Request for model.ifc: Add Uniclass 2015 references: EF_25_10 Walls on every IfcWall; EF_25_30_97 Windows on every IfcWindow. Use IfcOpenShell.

First a look at what the model holds.

```python
import ifcopenshell

model = ifcopenshell.open("model.ifc")
print(model.schema)
print("classifications:", [c.Name for c in model.by_type("IfcClassification")])
for ifc_class in ("IfcDoor", "IfcRoof", "IfcStair", "IfcWall", "IfcWindow"):
    print(ifc_class, len(model.by_type(ifc_class)))
```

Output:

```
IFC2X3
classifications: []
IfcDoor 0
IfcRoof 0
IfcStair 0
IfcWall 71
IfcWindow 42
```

```python
import ifcopenshell
import ifcopenshell.api.classification

model = ifcopenshell.open("model.ifc")

# IFC2X3 requires Source and Edition and has no link from the project to the system.
system = model.create_entity("IfcClassification", Source="NBS", Edition="2015", Name="Uniclass 2015")

codes = {
    "IfcWall": ("EF_25_10", "Walls"),
    "IfcWindow": ("EF_25_30_97", "Windows"),
}
for ifc_class, (code, name) in codes.items():
    products = model.by_type(ifc_class)
    ifcopenshell.api.classification.add_reference(
        model, products=products, classification=system, identification=code, name=name
    )
    print(code, len(products))

model.write("model_rev.ifc")
```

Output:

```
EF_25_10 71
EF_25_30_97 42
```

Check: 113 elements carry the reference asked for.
